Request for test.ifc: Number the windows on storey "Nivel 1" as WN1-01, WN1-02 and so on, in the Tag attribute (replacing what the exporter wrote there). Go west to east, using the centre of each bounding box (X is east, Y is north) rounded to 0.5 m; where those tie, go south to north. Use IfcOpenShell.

First a look at what the model holds.

```python
import ifcopenshell
import ifcopenshell.util.element
import ifcopenshell.util.placement

model = ifcopenshell.open("test.ifc")
print(model.schema)
storey = next(s for s in model.by_type("IfcBuildingStorey") if s.Name == "Nivel 1")
windows = [e for e in ifcopenshell.util.element.get_decomposition(storey) if e.is_a("IfcWindow")]
for e in sorted(windows, key=lambda e: e.id()):
    origin = ifcopenshell.util.placement.get_local_placement(e.ObjectPlacement)[:3, 3]
    print(e.id(), e.Tag, e.Name, origin.round(2) + 0.0, sep=" | ")
```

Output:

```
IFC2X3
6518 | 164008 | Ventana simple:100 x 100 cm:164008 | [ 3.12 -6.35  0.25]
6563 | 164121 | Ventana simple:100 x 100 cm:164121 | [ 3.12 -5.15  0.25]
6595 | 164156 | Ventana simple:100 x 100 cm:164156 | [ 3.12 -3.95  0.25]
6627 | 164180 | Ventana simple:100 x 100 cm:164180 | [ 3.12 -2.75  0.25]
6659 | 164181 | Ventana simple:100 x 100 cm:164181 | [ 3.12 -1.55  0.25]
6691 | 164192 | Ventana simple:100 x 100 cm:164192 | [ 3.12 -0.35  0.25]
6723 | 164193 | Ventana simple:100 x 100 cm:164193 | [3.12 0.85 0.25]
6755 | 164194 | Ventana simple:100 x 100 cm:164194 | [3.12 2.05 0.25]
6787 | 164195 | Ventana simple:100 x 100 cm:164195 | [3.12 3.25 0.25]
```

```python
import ifcopenshell
import ifcopenshell.geom
import ifcopenshell.util.element
import ifcopenshell.util.shape

model = ifcopenshell.open("test.ifc")
settings = ifcopenshell.geom.settings()
settings.set("use-world-coords", True)


def centre(element):
    shape = ifcopenshell.geom.create_shape(settings, element)
    return ifcopenshell.util.shape.get_bbox_centroid(shape.geometry)


storey = next(s for s in model.by_type("IfcBuildingStorey") if s.Name == "Nivel 1")
windows = [e for e in ifcopenshell.util.element.get_decomposition(storey) if e.is_a("IfcWindow")]

# Insertion points can sit at a corner or the storey origin, so sort by the geometry (in metres).
centres = {e: centre(e) for e in windows}
windows.sort(key=lambda e: (round(centres[e][0] / 0.5), centres[e][1]))

for i, e in enumerate(windows, start=1):
    number = f"WN1-{i:02d}"
    e.Tag = number
    print(e.id(), number)

model.write("test_updated.ifc")
```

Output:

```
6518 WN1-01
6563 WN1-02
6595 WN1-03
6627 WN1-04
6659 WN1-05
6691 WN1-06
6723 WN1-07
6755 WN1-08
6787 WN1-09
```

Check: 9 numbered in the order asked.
